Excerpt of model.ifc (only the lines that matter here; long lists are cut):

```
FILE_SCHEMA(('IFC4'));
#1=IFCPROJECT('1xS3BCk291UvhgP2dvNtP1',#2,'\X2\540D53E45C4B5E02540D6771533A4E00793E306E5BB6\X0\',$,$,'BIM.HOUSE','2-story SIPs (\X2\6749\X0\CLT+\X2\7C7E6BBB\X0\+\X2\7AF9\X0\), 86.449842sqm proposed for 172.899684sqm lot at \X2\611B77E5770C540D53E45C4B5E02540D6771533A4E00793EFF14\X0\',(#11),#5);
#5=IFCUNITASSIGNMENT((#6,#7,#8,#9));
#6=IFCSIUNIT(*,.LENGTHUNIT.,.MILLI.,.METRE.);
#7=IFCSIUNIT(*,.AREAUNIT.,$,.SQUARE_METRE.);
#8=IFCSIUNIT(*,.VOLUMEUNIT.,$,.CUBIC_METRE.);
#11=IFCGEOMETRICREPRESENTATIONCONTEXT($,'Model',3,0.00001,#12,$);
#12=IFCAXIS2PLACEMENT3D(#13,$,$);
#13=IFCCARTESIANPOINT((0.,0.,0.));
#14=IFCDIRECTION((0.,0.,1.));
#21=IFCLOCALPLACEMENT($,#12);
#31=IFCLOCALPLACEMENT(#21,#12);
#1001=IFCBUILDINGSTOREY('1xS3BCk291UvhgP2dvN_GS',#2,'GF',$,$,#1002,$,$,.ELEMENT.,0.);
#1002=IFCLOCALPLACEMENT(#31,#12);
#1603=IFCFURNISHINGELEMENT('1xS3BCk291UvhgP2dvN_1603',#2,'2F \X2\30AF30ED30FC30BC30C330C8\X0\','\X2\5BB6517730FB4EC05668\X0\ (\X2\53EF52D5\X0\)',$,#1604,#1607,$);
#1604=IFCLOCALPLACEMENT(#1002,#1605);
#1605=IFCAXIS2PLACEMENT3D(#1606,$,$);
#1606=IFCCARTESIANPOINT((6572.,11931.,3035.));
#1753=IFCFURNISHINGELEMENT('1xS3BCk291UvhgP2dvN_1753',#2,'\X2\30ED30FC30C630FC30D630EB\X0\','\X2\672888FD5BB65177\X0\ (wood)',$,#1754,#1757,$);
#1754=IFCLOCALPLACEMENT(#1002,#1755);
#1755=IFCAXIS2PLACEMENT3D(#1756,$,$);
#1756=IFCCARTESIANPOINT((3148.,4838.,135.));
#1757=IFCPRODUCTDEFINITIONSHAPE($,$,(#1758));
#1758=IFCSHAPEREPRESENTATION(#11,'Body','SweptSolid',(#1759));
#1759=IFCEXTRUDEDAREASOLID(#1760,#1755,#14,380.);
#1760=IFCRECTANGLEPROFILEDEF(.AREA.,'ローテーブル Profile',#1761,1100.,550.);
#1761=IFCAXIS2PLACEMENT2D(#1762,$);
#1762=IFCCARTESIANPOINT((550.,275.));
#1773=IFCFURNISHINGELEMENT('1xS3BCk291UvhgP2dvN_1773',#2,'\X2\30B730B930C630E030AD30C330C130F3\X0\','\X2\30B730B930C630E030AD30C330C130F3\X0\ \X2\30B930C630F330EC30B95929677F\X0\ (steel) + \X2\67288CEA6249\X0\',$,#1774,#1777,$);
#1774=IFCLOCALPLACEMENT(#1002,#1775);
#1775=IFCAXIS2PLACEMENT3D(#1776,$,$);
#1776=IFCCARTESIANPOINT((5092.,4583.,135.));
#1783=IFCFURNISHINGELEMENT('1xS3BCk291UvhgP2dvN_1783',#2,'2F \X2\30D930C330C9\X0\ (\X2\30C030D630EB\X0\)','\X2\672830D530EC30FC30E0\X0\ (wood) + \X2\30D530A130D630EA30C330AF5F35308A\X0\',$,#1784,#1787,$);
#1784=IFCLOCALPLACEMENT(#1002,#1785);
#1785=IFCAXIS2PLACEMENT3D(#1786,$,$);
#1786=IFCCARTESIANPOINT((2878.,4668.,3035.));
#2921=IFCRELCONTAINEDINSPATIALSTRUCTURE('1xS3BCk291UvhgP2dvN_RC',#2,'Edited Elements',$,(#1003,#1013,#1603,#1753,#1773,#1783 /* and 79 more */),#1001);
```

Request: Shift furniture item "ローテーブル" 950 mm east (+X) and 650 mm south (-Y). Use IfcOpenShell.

```python
import ifcopenshell
import ifcopenshell.api.geometry
import ifcopenshell.util.placement
import ifcopenshell.util.unit

model = ifcopenshell.open("model.ifc")
unit_scale = ifcopenshell.util.unit.calculate_unit_scale(model)

item = model.by_guid("1xS3BCk291UvhgP2dvN_1753")
matrix = ifcopenshell.util.placement.get_local_placement(item.ObjectPlacement)
matrix[0, 3] += 0.95 / unit_scale
matrix[1, 3] -= 0.65 / unit_scale
ifcopenshell.api.geometry.edit_object_placement(model, product=item, matrix=matrix, is_si=False)

print(ifcopenshell.util.placement.get_local_placement(item.ObjectPlacement).round(3) + 0.0)

model.write("model_updated.ifc")
```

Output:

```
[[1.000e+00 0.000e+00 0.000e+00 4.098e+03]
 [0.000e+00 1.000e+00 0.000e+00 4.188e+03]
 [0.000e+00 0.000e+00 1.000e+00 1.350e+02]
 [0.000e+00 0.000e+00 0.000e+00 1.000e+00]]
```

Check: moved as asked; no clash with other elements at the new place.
